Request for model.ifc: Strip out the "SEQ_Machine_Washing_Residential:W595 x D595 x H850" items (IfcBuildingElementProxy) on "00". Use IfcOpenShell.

First a look at what the model holds.

```python
import ifcopenshell
import ifcopenshell.util.element

model = ifcopenshell.open("model.ifc")
print(model.schema)
storey = next(s for s in model.by_type("IfcBuildingStorey") if s.Name == "00")
proxies = [e for e in ifcopenshell.util.element.get_decomposition(storey) if e.is_a("IfcBuildingElementProxy")]
seen = {}
for e in proxies:
    element_type = ifcopenshell.util.element.get_type(e)
    name = element_type.Name if element_type not in (None, e) else None
    seen[name] = seen.get(name, 0) + 1
for name, count in sorted(seen.items(), key=str):
    print(count, "x", name)
```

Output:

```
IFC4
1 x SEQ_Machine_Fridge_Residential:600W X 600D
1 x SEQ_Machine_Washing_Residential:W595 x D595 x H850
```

```python
import ifcopenshell
import ifcopenshell.api.root
import ifcopenshell.util.element

model = ifcopenshell.open("model.ifc")

storey = next(s for s in model.by_type("IfcBuildingStorey") if s.Name == "00")
proxies = [e for e in ifcopenshell.util.element.get_decomposition(storey) if e.is_a("IfcBuildingElementProxy")]
targets = [e for e in proxies if (t := ifcopenshell.util.element.get_type(e)) not in (None, e) and t.Name == "SEQ_Machine_Washing_Residential:W595 x D595 x H850"]

for e in targets:
    ifcopenshell.api.root.remove_product(model, product=e)
print(len(targets), "removed")

model.write("model_updated.ifc")
```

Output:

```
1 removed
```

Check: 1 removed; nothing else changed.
